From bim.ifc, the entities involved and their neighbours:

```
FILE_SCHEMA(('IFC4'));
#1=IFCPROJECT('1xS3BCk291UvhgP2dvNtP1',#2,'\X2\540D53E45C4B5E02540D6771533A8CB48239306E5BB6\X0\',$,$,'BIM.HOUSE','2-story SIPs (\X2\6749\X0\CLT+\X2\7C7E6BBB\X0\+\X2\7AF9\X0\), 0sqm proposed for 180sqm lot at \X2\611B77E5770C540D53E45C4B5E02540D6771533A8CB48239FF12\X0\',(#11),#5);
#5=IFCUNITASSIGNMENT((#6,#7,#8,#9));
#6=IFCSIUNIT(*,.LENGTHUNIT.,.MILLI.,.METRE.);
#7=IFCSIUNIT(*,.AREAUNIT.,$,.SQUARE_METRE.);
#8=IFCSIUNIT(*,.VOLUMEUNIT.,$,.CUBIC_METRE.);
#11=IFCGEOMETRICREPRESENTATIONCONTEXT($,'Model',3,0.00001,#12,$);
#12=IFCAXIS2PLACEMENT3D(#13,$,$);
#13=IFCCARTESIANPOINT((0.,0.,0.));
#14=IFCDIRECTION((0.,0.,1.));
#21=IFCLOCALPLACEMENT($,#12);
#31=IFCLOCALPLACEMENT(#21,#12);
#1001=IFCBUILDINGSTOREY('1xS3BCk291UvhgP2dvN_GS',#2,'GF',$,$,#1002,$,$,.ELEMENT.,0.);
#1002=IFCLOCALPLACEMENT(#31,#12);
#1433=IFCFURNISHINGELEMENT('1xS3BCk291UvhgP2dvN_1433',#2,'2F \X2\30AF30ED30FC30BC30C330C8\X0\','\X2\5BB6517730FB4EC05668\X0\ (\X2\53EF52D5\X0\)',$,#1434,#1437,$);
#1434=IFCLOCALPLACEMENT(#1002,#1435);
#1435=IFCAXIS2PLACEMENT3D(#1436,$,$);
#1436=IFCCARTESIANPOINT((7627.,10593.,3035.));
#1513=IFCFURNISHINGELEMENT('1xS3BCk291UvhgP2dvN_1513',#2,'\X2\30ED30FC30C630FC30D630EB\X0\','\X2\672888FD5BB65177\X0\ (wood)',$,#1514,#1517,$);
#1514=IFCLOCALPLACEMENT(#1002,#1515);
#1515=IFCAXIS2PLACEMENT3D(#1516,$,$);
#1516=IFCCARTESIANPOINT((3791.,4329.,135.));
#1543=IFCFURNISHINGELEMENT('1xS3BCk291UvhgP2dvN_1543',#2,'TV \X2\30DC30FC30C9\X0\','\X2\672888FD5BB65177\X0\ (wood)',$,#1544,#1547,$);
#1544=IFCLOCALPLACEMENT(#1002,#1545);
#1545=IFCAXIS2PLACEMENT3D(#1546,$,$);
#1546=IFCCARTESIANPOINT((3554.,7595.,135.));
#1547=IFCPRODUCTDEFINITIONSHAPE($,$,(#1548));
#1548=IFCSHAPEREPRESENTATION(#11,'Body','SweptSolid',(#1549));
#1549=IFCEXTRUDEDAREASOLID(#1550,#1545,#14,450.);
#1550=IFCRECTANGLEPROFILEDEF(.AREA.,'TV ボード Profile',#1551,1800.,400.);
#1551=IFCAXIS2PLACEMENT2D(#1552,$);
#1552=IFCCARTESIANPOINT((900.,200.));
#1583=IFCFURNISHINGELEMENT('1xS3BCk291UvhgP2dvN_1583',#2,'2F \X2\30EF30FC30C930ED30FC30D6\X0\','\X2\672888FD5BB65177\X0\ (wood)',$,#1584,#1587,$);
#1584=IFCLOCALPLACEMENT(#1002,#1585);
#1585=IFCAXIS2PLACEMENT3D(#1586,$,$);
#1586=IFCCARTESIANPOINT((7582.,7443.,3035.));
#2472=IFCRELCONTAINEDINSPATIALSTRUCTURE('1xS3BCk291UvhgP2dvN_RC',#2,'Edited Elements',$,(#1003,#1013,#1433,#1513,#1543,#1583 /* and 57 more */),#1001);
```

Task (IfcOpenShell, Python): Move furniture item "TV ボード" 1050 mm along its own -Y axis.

```python
import ifcopenshell
import ifcopenshell.api.geometry
import ifcopenshell.util.placement

model = ifcopenshell.open("bim.ifc")

item = model.by_id(1543)
matrix = ifcopenshell.util.placement.get_local_placement(item.ObjectPlacement)
matrix[:3, 3] -= matrix[:3, 1] * 1050.0
ifcopenshell.api.geometry.edit_object_placement(model, product=item, matrix=matrix, is_si=False)

print(ifcopenshell.util.placement.get_local_placement(item.ObjectPlacement).round(3) + 0.0)

model.write("bim-out.ifc")
```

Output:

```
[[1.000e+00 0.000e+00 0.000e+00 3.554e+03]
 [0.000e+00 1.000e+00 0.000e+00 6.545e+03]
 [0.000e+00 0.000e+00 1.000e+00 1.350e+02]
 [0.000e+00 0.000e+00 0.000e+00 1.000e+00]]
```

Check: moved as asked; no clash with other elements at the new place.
